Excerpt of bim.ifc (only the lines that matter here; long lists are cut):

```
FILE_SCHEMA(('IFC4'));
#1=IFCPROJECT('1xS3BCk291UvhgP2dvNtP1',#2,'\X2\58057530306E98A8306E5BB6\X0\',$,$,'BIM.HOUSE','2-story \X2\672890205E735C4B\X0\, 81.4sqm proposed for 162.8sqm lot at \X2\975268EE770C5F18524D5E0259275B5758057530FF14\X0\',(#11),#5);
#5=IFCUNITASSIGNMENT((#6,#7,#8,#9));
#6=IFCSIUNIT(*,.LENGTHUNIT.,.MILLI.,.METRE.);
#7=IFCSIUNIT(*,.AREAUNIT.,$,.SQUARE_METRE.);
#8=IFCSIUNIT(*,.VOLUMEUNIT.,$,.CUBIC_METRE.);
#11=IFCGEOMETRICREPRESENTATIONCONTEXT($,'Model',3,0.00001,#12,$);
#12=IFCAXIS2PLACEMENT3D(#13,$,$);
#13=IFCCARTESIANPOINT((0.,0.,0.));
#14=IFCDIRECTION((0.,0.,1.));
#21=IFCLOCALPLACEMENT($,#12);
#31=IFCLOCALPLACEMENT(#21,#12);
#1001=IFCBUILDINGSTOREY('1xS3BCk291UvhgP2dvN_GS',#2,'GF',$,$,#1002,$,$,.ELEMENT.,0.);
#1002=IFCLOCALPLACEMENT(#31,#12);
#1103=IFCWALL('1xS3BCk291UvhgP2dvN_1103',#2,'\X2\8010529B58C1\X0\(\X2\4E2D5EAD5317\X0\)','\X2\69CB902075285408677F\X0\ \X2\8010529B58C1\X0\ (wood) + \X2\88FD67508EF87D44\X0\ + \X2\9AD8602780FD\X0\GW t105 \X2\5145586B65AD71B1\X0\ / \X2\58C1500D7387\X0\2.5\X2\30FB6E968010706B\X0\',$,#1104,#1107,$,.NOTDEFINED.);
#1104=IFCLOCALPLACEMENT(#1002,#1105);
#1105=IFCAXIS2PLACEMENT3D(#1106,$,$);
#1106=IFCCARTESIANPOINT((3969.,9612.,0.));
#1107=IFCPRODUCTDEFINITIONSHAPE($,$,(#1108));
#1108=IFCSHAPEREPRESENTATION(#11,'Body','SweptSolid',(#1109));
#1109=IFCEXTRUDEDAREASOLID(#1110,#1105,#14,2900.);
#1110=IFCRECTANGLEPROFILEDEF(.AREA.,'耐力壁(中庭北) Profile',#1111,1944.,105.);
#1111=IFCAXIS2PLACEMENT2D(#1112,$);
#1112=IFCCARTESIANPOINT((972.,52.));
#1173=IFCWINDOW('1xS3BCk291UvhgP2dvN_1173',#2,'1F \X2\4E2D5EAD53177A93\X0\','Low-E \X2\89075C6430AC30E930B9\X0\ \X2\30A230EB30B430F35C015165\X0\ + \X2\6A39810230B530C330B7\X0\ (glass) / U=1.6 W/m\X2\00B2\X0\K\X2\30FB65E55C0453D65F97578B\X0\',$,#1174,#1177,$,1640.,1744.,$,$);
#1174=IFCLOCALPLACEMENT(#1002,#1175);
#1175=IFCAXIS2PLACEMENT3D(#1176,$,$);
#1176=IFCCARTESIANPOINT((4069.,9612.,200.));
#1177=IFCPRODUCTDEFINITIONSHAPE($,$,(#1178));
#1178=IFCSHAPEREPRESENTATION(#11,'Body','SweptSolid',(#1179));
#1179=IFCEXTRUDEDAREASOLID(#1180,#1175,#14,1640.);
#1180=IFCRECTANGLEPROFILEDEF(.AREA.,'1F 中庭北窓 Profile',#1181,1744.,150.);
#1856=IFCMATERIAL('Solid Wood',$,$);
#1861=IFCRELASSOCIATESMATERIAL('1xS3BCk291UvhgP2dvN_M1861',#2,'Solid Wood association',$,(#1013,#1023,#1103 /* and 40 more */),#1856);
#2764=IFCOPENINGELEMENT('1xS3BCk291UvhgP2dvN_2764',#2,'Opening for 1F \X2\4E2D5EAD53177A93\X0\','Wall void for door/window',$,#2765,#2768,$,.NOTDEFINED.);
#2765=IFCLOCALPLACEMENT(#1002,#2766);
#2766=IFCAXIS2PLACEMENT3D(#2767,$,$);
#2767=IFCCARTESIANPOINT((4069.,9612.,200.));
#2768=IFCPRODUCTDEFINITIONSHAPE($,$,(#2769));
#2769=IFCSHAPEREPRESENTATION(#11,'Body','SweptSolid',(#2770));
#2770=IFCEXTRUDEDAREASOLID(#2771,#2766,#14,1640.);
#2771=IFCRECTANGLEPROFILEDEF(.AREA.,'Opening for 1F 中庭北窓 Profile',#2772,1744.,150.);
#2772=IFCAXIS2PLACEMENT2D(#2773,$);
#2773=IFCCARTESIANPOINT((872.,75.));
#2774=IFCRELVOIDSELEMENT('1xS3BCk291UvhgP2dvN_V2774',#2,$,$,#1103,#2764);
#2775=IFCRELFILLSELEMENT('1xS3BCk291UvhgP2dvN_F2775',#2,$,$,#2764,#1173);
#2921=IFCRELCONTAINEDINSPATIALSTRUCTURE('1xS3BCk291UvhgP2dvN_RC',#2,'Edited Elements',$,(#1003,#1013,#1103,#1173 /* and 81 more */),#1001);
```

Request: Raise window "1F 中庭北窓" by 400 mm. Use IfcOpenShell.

```python
import numpy as np
import ifcopenshell
import ifcopenshell.api.geometry
import ifcopenshell.util.placement
import ifcopenshell.util.unit

model = ifcopenshell.open("bim.ifc")
unit_scale = ifcopenshell.util.unit.calculate_unit_scale(model)

window = model.by_guid("1xS3BCk291UvhgP2dvN_1173")
opening = window.FillsVoids[0].RelatingOpeningElement
dz = 0.4 / unit_scale

shift = np.array([0.0, 0.0, dz])
# The window is not placed relative to its opening, so move both.
for product in (opening, window):
    matrix = ifcopenshell.util.placement.get_local_placement(product.ObjectPlacement)
    matrix[:3, 3] += shift
    ifcopenshell.api.geometry.edit_object_placement(model, product=product, matrix=matrix, is_si=False)

print(f"moved by {dz * unit_scale:+.3f} m")

model.write("bim_v2.ifc")
```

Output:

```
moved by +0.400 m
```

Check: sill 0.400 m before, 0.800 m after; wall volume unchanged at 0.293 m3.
